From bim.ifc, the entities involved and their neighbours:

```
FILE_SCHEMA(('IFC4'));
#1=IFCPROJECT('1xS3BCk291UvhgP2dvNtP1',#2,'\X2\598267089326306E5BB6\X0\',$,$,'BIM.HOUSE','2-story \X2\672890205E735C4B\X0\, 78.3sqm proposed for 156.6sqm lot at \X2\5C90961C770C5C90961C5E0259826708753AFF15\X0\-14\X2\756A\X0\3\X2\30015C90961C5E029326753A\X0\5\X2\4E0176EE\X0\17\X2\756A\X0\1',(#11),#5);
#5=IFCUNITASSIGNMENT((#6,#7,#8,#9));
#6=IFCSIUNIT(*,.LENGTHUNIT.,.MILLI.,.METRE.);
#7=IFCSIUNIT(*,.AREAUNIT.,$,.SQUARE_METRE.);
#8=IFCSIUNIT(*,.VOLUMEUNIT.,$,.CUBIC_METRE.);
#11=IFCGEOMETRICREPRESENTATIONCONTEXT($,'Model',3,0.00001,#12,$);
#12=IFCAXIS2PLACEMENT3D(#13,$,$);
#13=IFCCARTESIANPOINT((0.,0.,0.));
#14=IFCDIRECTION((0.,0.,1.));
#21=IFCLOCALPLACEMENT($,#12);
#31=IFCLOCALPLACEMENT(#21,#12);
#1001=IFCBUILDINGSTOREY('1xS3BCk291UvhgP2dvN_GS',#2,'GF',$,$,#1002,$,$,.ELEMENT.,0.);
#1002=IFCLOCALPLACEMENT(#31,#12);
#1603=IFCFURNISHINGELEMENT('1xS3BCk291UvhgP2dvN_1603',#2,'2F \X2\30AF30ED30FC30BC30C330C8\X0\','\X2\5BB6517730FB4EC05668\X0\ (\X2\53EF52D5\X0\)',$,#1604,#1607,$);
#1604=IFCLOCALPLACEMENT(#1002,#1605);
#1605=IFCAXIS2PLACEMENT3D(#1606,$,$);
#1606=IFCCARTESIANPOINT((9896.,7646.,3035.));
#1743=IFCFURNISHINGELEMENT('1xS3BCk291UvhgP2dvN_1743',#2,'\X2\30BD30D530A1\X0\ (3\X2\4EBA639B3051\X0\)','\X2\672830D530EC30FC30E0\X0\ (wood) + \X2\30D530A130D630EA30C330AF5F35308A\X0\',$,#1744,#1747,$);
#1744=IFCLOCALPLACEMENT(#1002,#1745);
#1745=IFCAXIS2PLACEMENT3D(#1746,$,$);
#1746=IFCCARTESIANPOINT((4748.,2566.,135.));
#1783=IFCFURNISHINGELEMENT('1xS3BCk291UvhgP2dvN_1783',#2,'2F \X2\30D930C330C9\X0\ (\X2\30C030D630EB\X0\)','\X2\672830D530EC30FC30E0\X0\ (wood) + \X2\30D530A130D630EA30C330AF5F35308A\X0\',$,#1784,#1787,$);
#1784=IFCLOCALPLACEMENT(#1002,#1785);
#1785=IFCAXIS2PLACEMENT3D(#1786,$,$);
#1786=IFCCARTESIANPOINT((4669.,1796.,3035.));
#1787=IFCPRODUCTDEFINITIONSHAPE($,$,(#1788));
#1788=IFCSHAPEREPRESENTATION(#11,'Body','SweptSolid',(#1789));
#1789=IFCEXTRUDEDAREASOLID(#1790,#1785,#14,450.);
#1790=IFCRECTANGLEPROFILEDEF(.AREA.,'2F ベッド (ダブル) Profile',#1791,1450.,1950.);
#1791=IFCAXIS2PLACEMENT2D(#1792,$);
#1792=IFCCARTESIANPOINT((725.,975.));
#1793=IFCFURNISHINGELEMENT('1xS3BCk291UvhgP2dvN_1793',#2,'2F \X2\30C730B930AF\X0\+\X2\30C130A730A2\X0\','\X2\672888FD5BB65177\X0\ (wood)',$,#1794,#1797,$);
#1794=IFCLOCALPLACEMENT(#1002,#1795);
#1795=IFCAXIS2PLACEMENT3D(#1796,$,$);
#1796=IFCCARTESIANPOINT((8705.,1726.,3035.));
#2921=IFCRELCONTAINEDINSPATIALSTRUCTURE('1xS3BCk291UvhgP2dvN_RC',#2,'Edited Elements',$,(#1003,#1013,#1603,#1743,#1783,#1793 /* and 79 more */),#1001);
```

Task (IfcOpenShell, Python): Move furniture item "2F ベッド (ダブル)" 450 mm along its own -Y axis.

```python
import ifcopenshell
import ifcopenshell.api.geometry
import ifcopenshell.util.placement

model = ifcopenshell.open("bim.ifc")

item = model.by_guid("1xS3BCk291UvhgP2dvN_1783")
matrix = ifcopenshell.util.placement.get_local_placement(item.ObjectPlacement)
matrix[:3, 3] -= matrix[:3, 1] * 450.0
ifcopenshell.api.geometry.edit_object_placement(model, product=item, matrix=matrix, is_si=False)

print(ifcopenshell.util.placement.get_local_placement(item.ObjectPlacement).round(3) + 0.0)

model.write("bim_edited.ifc")
```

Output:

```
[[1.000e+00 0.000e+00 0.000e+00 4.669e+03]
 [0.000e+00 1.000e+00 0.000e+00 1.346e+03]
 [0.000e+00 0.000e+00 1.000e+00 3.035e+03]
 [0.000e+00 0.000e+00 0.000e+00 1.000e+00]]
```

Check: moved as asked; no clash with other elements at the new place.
